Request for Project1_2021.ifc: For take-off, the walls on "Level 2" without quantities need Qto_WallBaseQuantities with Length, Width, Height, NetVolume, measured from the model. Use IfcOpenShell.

First a look at what the model holds.

```python
import ifcopenshell
import ifcopenshell.util.element
import ifcopenshell.util.unit

model = ifcopenshell.open("Project1_2021.ifc")
print(model.schema)
for unit_type in ("LENGTHUNIT", "AREAUNIT", "VOLUMEUNIT"):
    print(unit_type, ifcopenshell.util.unit.calculate_unit_scale(model, unit_type))
storey = next(s for s in model.by_type("IfcBuildingStorey") if s.Name == "Level 2")
walls = [e for e in ifcopenshell.util.element.get_decomposition(storey) if e.is_a("IfcWall")]
for e in sorted(walls, key=lambda e: e.id()):
    print(e.id(), e.is_a(), e.Name, list(ifcopenshell.util.element.get_psets(e, qtos_only=True)), sep=" | ")
```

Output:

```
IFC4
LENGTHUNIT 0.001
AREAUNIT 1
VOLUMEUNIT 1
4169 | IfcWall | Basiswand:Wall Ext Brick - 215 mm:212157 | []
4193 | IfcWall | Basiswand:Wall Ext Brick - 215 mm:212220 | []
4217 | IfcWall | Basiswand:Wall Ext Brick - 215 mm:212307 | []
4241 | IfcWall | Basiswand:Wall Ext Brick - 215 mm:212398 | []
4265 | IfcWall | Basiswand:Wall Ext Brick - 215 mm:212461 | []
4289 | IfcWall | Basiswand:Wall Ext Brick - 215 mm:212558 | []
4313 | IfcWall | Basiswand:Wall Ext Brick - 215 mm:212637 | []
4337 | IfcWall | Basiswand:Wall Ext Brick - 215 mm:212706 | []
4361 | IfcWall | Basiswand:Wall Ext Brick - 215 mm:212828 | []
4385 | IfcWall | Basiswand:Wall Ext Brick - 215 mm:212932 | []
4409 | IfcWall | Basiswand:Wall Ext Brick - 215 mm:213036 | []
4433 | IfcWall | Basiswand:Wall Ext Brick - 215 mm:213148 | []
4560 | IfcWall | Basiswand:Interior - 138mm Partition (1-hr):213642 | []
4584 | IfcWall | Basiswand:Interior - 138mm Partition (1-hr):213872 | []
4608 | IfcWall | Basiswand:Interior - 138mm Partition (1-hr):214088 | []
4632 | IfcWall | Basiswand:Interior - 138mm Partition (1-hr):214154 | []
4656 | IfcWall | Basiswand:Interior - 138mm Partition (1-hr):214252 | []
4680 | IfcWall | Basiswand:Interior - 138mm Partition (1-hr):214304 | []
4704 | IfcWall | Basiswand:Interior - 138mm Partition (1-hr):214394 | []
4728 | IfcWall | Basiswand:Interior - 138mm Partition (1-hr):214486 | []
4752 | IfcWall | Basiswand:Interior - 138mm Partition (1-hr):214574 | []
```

```python
import ifcopenshell
import ifcopenshell.api.pset
import ifcopenshell.geom
import ifcopenshell.util.element
import ifcopenshell.util.shape
import ifcopenshell.util.unit

model = ifcopenshell.open("Project1_2021.ifc")
unit_scale = ifcopenshell.util.unit.calculate_unit_scale(model)
volume_scale = ifcopenshell.util.unit.calculate_unit_scale(model, "VOLUMEUNIT")
settings = ifcopenshell.geom.settings()

storey = next(s for s in model.by_type("IfcBuildingStorey") if s.Name == "Level 2")
walls = [e for e in ifcopenshell.util.element.get_decomposition(storey) if e.is_a("IfcWall")]

for e in sorted(walls, key=lambda e: e.id()):
    if ifcopenshell.util.element.get_psets(e, qtos_only=True, should_inherit=False):
        continue
    # Geometry comes back in metres, in the element's own axes.
    shape = ifcopenshell.geom.create_shape(settings, e)
    values = {
        "Length": ifcopenshell.util.shape.get_x(shape.geometry) / unit_scale,
        "Width": ifcopenshell.util.shape.get_y(shape.geometry) / unit_scale,
        "Height": ifcopenshell.util.shape.get_z(shape.geometry) / unit_scale,
        "NetVolume": ifcopenshell.util.shape.get_volume(shape.geometry) / volume_scale,
    }
    qto = ifcopenshell.api.pset.add_qto(model, product=e, name="Qto_WallBaseQuantities")
    ifcopenshell.api.pset.edit_qto(model, qto=qto, properties=values)
    print(e.id(), {k: round(v, 3) for k, v in values.items()})

model.write("Project1_2021_rev.ifc")
```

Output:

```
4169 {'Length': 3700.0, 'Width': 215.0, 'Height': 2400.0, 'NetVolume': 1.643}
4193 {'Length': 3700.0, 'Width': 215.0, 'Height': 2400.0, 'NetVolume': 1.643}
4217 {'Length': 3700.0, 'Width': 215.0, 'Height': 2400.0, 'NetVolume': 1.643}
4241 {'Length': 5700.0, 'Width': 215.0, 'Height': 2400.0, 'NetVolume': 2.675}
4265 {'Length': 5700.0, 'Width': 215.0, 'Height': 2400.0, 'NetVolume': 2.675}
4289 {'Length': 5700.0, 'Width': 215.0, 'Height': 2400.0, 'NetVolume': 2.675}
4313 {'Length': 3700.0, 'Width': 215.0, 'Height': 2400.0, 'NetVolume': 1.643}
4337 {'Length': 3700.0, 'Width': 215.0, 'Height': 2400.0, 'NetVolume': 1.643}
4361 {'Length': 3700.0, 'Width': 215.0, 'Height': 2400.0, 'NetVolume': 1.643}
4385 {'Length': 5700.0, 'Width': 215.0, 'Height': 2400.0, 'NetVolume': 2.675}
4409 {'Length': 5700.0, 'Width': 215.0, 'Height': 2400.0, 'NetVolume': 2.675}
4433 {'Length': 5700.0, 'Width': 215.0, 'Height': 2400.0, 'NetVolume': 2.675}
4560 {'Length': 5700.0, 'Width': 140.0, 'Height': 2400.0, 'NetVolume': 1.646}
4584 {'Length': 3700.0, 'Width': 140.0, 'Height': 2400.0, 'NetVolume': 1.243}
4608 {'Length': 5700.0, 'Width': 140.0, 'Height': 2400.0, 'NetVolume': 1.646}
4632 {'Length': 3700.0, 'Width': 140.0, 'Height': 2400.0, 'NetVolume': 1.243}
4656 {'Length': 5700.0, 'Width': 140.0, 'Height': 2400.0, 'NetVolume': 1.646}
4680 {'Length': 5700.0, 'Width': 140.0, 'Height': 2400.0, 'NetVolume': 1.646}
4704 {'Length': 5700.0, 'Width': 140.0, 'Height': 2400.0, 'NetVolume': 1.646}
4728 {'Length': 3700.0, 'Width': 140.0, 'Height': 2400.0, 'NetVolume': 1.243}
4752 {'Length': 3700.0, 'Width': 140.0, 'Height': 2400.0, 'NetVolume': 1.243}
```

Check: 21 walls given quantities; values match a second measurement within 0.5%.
